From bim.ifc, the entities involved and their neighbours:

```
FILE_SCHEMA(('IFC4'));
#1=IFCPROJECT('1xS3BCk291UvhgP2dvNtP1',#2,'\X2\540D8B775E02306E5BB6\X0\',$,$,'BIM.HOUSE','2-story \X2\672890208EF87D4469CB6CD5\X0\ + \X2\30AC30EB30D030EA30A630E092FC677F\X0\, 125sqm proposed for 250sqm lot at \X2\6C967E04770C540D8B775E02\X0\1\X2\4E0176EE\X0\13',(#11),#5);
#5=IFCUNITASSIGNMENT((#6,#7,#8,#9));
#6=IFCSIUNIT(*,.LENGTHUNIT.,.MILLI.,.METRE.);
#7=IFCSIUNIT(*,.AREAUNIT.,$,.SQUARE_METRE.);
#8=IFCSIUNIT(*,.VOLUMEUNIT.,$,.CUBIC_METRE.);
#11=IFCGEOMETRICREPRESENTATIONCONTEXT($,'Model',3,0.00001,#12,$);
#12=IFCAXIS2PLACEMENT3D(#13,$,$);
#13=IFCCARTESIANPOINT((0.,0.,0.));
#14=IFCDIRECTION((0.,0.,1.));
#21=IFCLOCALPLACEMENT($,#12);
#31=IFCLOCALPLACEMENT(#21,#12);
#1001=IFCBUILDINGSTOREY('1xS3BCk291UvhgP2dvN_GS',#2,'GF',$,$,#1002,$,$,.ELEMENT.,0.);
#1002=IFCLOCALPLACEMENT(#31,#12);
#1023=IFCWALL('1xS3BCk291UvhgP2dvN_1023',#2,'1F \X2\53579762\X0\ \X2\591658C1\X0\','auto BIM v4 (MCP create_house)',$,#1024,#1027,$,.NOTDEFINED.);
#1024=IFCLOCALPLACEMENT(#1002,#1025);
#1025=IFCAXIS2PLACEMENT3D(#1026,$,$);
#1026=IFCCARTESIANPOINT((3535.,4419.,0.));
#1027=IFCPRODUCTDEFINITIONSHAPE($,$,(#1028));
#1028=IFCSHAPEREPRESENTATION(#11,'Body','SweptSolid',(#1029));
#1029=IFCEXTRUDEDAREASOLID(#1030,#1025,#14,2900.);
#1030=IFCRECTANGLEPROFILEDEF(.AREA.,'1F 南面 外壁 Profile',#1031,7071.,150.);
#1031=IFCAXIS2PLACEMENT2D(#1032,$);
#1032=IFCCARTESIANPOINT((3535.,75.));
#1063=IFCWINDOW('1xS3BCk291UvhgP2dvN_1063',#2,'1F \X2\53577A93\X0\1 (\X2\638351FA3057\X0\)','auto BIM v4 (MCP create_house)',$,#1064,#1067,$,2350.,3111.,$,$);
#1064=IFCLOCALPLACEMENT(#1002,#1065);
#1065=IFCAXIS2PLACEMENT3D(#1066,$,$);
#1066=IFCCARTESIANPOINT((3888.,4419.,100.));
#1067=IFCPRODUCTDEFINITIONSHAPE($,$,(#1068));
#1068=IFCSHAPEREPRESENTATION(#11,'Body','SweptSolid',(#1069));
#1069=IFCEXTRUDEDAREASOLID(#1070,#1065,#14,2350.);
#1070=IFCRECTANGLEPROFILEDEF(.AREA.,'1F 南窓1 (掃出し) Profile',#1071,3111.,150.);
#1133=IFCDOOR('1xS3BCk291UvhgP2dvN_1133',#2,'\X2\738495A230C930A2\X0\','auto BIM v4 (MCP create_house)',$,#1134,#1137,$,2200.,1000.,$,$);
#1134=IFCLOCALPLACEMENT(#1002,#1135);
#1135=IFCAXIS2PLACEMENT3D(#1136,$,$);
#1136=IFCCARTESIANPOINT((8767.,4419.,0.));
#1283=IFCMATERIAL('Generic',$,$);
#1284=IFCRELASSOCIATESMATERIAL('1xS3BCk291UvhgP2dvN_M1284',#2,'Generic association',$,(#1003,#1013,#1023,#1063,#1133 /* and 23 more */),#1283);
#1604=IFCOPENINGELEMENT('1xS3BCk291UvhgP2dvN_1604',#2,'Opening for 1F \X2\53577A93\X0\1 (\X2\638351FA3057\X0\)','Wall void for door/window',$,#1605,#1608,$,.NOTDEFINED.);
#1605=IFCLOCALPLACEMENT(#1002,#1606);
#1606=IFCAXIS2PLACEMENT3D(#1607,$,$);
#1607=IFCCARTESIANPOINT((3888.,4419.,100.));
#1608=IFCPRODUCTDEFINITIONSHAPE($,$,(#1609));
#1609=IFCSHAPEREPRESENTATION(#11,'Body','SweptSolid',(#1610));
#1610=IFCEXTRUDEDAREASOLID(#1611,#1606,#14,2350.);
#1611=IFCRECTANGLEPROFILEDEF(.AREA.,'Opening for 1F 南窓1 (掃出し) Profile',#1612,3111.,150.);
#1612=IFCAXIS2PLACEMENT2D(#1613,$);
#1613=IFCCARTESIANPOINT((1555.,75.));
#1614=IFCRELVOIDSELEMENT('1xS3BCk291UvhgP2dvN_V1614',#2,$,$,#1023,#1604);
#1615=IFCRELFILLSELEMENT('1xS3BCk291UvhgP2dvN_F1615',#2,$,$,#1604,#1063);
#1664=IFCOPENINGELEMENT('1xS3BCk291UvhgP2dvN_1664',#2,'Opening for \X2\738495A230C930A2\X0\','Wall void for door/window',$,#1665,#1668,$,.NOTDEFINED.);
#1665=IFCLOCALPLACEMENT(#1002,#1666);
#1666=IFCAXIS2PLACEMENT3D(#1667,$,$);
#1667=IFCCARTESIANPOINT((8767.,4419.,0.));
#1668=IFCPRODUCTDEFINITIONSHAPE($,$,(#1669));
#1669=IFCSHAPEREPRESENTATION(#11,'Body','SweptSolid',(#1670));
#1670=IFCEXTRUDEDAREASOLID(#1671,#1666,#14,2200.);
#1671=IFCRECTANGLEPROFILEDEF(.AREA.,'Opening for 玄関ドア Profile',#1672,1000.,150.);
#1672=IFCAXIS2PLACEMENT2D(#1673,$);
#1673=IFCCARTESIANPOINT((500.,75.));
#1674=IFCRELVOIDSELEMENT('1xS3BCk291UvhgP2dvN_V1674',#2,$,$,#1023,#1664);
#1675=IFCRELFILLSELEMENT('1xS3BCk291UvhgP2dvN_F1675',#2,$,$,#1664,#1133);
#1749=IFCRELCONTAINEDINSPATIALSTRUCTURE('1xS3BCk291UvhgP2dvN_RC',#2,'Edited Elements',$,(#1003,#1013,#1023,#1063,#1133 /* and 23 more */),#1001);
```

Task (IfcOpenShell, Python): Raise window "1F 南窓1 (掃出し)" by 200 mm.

```python
import numpy as np
import ifcopenshell
import ifcopenshell.api.geometry
import ifcopenshell.util.placement
import ifcopenshell.util.unit

model = ifcopenshell.open("bim.ifc")
unit_scale = ifcopenshell.util.unit.calculate_unit_scale(model)

window = model.by_guid("1xS3BCk291UvhgP2dvN_1063")
opening = window.FillsVoids[0].RelatingOpeningElement
dz = 200.0

shift = np.array([0.0, 0.0, dz])
# The window is not placed relative to its opening, so move both.
for product in (opening, window):
    matrix = ifcopenshell.util.placement.get_local_placement(product.ObjectPlacement)
    matrix[:3, 3] += shift
    ifcopenshell.api.geometry.edit_object_placement(model, product=product, matrix=matrix, is_si=False)

print(f"moved by {dz * unit_scale:+.3f} m")

model.write("bim_rev.ifc")
```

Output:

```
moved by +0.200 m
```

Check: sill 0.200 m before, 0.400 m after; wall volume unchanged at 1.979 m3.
